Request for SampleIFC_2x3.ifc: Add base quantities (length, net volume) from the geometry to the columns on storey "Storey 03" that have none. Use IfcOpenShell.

First a look at what the model holds.

```python
import ifcopenshell
import ifcopenshell.util.element
import ifcopenshell.util.unit

model = ifcopenshell.open("SampleIFC_2x3.ifc")
print(model.schema)
for unit_type in ("LENGTHUNIT", "AREAUNIT", "VOLUMEUNIT"):
    print(unit_type, ifcopenshell.util.unit.calculate_unit_scale(model, unit_type))
storey = next(s for s in model.by_type("IfcBuildingStorey") if s.Name == "Storey 03")
columns = [e for e in ifcopenshell.util.element.get_decomposition(storey) if e.is_a("IfcColumn")]
for e in sorted(columns, key=lambda e: e.id()):
    print(e.id(), e.is_a(), e.Name, list(ifcopenshell.util.element.get_psets(e, qtos_only=True)), sep=" | ")
```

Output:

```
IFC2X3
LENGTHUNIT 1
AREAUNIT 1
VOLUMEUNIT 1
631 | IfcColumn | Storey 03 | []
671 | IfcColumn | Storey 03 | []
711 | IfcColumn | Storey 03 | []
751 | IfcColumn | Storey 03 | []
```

```python
import ifcopenshell
import ifcopenshell.api.pset
import ifcopenshell.geom
import ifcopenshell.util.element
import ifcopenshell.util.shape
import ifcopenshell.util.unit

model = ifcopenshell.open("SampleIFC_2x3.ifc")
unit_scale = ifcopenshell.util.unit.calculate_unit_scale(model)
volume_scale = ifcopenshell.util.unit.calculate_unit_scale(model, "VOLUMEUNIT")
settings = ifcopenshell.geom.settings()

storey = next(s for s in model.by_type("IfcBuildingStorey") if s.Name == "Storey 03")
columns = [e for e in ifcopenshell.util.element.get_decomposition(storey) if e.is_a("IfcColumn")]

for e in sorted(columns, key=lambda e: e.id()):
    if ifcopenshell.util.element.get_psets(e, qtos_only=True, should_inherit=False):
        continue
    # Geometry comes back in metres, in the element's own axes.
    shape = ifcopenshell.geom.create_shape(settings, e)
    values = {
        "Length": ifcopenshell.util.shape.get_z(shape.geometry) / unit_scale,
        "NetVolume": ifcopenshell.util.shape.get_volume(shape.geometry) / volume_scale,
    }
    qto = ifcopenshell.api.pset.add_qto(model, product=e, name="BaseQuantities")
    ifcopenshell.api.pset.edit_qto(model, qto=qto, properties=values)
    print(e.id(), {k: round(v, 3) for k, v in values.items()})

model.write("SampleIFC_2x3_edited.ifc")
```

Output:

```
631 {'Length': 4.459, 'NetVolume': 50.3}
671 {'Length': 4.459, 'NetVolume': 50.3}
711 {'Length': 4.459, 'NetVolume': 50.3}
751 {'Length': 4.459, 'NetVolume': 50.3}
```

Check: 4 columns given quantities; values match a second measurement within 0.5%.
